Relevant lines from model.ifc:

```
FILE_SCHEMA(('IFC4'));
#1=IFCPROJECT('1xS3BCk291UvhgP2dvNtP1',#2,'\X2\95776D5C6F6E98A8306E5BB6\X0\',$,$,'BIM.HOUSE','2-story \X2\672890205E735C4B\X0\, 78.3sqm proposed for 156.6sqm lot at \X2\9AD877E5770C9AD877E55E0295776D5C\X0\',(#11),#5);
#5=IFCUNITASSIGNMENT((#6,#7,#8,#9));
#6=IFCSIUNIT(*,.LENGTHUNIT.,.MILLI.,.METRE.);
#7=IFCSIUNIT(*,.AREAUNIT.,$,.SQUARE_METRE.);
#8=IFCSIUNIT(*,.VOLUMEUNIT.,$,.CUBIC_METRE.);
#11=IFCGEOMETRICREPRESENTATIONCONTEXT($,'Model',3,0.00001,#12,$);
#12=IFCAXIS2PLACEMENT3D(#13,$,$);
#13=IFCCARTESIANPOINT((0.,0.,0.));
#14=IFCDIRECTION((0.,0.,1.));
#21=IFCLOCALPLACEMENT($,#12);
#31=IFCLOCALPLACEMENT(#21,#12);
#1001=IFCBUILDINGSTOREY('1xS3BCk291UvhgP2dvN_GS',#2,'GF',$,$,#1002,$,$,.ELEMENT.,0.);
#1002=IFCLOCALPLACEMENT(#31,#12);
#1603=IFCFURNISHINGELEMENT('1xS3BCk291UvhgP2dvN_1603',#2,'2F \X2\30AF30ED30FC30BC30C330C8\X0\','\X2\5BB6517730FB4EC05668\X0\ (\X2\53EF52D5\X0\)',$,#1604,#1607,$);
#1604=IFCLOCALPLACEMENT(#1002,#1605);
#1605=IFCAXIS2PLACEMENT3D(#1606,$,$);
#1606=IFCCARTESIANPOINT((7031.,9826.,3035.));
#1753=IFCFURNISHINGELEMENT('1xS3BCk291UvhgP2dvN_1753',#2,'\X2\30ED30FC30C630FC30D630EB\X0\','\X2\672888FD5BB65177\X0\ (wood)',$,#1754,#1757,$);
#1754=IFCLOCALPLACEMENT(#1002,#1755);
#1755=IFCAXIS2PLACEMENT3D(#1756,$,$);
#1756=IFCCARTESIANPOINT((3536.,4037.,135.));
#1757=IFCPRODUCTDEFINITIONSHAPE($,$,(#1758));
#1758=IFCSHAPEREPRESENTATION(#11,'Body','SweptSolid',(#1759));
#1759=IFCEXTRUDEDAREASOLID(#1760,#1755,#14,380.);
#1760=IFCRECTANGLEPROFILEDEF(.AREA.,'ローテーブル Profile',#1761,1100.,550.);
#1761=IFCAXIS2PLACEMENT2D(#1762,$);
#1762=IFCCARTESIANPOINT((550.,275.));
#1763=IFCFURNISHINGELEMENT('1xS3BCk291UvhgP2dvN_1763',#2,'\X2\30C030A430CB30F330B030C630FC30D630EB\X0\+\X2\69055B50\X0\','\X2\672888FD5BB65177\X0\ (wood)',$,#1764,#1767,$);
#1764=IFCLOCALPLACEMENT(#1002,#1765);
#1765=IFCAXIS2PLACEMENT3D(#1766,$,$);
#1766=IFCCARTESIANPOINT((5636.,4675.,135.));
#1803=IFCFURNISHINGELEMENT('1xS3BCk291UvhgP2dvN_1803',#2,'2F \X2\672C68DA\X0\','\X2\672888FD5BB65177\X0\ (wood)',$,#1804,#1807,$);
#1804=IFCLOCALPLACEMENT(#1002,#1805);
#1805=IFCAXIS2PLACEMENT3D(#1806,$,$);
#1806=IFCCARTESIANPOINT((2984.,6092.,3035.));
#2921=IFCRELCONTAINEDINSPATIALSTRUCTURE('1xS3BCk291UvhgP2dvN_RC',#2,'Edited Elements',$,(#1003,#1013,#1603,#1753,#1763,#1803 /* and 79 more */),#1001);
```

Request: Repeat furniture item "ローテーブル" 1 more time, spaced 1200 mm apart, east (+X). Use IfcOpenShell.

```python
import numpy as np
import ifcopenshell
import ifcopenshell.api.geometry
import ifcopenshell.api.root
import ifcopenshell.util.element
import ifcopenshell.util.placement
import ifcopenshell.util.unit

model = ifcopenshell.open("model.ifc")
unit_scale = ifcopenshell.util.unit.calculate_unit_scale(model)


def reuse_history(source, copy):
    """copy_class also copies each property set's owner history, people and application; keep the originals."""
    for rel in copy.IsDefinedBy:
        if rel.is_a("IfcRelDefinesByProperties") and (history := rel.RelatingPropertyDefinition.OwnerHistory):
            rel.RelatingPropertyDefinition.OwnerHistory = source.OwnerHistory
            ifcopenshell.util.element.remove_deep2(model, history)


source = model.by_guid("1xS3BCk291UvhgP2dvN_1753")
base = ifcopenshell.util.placement.get_local_placement(source.ObjectPlacement)
step = np.array([1.0, 0.0, 0.0]) * 1.2 / unit_scale

for i in range(1, 2):
    copy = ifcopenshell.api.root.copy_class(model, product=source)
    copy.Representation = ifcopenshell.util.element.copy_deep(
        model, source.Representation, exclude=["IfcGeometricRepresentationContext", "IfcRepresentationMap"]
    )
    reuse_history(source, copy)
    matrix = base.copy()
    matrix[:3, 3] += i * step
    print("added at", matrix[:3, 3].round(3) + 0.0)
    ifcopenshell.api.geometry.edit_object_placement(model, product=copy, matrix=matrix, is_si=False)

model.write("model_edited.ifc")
```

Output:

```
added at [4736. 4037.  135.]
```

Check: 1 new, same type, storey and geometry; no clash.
